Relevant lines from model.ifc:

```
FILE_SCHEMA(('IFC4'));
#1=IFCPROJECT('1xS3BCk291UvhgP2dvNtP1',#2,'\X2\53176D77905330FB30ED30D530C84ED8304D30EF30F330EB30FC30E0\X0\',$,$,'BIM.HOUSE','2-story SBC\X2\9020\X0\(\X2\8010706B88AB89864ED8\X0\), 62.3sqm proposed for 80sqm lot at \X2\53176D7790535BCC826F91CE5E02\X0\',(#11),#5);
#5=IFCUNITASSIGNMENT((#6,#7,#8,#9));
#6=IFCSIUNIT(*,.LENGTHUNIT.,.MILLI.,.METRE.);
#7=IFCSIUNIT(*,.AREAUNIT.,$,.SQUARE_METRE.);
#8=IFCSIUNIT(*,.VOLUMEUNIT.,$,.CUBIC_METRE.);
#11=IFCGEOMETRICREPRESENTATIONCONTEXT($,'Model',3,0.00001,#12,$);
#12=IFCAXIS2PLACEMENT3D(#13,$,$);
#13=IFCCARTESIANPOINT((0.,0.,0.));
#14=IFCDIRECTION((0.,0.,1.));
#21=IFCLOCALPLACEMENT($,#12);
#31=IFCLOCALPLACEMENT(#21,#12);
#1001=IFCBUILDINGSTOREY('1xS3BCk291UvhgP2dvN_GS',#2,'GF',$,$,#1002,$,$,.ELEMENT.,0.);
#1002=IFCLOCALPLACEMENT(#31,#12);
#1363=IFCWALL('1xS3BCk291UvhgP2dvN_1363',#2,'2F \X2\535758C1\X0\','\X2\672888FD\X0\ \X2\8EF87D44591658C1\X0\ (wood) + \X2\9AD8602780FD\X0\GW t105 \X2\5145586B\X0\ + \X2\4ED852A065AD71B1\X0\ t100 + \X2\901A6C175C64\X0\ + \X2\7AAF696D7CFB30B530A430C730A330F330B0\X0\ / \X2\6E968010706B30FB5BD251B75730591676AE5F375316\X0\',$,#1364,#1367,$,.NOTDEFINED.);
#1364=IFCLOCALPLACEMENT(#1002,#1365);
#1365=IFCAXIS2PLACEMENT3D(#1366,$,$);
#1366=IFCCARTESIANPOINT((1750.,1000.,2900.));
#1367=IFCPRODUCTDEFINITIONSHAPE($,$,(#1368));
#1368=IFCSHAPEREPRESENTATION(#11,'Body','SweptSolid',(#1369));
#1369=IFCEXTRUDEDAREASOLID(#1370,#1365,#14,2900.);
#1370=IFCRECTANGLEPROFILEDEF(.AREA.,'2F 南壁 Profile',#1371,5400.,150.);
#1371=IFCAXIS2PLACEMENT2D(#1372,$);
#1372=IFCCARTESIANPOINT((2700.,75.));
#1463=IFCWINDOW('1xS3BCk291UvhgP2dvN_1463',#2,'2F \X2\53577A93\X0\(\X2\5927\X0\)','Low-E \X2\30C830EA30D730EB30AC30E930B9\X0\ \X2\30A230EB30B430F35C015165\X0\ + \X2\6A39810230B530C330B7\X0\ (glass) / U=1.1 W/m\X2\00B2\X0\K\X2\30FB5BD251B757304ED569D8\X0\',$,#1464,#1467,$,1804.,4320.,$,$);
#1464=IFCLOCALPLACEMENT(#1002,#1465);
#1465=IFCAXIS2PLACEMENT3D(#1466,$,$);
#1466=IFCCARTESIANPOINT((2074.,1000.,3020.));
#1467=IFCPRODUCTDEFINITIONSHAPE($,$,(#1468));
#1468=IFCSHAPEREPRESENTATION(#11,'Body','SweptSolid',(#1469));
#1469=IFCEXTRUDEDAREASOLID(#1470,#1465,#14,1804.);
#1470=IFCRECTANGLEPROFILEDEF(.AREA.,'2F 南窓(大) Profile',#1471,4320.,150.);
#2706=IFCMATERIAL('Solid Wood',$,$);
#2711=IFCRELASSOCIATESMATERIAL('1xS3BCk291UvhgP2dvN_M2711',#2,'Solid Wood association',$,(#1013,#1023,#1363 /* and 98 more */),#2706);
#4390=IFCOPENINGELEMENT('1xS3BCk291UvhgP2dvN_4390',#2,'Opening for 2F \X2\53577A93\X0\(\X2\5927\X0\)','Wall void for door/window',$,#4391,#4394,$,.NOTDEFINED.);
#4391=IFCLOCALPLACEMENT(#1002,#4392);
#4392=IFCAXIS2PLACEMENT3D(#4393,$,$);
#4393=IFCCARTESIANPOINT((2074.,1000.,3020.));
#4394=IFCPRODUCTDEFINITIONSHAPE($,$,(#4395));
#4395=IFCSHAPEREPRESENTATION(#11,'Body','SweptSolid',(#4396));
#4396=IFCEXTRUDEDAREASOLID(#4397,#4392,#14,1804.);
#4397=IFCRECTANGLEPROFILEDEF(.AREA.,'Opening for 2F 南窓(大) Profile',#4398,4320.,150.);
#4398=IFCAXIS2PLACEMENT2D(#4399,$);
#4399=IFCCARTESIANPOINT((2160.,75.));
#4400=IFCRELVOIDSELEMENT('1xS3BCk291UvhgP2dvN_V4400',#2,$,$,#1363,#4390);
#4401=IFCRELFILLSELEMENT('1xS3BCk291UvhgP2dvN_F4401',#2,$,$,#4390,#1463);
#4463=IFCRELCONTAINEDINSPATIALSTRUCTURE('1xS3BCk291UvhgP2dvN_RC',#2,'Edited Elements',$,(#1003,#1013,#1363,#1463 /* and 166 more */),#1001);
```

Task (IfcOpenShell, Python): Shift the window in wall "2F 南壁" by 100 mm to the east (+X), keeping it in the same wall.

```python
import ifcopenshell
import ifcopenshell.api.geometry
import ifcopenshell.util.placement

model = ifcopenshell.open("model.ifc")

window = model.by_id(1463)
opening = window.FillsVoids[0].RelatingOpeningElement
wall = opening.VoidsElements[0].RelatingBuildingElement

wall_matrix = ifcopenshell.util.placement.get_local_placement(wall.ObjectPlacement)
shift = wall_matrix[:3, 0] * 100.0
before = ifcopenshell.util.placement.get_local_placement(window.ObjectPlacement)[:3, 3].copy()

# The window is not placed relative to its opening, so move both.
for product in (opening, window):
    matrix = ifcopenshell.util.placement.get_local_placement(product.ObjectPlacement)
    matrix[:3, 3] += shift
    ifcopenshell.api.geometry.edit_object_placement(model, product=product, matrix=matrix, is_si=False)

after = ifcopenshell.util.placement.get_local_placement(window.ObjectPlacement)[:3, 3]
print("window moved by", (after - before).round(3) + 0.0)

model.write("model_v2.ifc")
```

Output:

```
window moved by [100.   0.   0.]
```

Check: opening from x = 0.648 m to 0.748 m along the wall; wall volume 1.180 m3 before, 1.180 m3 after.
